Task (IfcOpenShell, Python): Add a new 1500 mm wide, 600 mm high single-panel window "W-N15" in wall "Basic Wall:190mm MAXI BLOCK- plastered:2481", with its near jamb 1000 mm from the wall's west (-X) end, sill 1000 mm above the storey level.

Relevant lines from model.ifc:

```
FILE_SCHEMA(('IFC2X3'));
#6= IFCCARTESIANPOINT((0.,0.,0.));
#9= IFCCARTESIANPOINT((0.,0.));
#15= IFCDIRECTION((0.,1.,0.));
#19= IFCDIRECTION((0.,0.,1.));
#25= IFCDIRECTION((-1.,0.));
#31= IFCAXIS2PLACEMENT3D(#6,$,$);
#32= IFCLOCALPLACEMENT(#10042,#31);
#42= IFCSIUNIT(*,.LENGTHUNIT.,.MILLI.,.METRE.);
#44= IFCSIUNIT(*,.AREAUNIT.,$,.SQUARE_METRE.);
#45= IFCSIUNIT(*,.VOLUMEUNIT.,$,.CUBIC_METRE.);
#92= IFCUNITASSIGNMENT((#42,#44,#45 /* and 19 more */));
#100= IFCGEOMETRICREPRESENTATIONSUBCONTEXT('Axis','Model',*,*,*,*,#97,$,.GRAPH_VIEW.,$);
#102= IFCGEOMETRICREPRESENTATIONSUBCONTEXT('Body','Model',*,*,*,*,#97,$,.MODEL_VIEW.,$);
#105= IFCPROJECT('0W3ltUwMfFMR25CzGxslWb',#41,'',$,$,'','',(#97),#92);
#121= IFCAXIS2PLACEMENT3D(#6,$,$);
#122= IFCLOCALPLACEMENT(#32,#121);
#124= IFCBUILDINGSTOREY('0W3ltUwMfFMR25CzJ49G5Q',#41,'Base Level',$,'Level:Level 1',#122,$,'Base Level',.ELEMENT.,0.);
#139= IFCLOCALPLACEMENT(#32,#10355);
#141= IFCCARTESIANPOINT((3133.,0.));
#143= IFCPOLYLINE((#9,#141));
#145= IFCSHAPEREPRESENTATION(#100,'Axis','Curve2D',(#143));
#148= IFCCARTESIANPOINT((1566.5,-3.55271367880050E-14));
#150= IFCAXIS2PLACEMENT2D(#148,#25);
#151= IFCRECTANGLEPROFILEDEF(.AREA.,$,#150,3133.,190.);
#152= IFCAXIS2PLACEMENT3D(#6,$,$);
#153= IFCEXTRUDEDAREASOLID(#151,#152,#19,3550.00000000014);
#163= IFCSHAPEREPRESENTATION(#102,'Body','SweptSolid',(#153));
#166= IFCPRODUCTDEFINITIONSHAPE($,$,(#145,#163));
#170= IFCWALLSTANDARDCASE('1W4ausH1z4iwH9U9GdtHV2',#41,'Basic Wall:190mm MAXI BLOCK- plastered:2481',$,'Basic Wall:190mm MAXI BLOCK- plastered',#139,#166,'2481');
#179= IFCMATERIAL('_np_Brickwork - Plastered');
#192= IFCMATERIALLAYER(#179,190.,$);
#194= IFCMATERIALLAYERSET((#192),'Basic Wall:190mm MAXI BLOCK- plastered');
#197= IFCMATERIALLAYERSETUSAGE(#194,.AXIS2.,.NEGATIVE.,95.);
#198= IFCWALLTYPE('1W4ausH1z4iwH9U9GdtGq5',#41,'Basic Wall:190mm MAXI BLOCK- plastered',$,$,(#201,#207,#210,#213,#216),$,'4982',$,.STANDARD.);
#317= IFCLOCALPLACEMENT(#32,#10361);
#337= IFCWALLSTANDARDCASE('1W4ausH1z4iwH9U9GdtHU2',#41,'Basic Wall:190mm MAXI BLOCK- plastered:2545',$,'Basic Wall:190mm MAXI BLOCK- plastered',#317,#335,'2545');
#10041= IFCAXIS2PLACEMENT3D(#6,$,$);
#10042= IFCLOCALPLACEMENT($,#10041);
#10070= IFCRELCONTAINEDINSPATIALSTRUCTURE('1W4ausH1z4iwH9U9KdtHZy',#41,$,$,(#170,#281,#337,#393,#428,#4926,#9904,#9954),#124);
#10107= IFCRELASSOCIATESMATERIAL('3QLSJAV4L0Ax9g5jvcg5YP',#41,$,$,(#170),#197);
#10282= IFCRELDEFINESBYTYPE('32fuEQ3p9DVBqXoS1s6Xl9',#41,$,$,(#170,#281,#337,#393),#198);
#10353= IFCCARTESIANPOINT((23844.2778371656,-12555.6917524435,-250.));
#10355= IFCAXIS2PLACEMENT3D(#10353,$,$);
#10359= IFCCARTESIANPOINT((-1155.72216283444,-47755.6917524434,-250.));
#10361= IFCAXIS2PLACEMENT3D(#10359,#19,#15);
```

```python
import numpy as np
import ifcopenshell
import ifcopenshell.api.feature
import ifcopenshell.api.geometry
import ifcopenshell.api.root
import ifcopenshell.api.spatial
import ifcopenshell.api.type
import ifcopenshell.geom
import ifcopenshell.util.element
import ifcopenshell.util.placement
import ifcopenshell.util.representation
import ifcopenshell.util.shape
import ifcopenshell.util.unit

model = ifcopenshell.open("model.ifc")
unit_scale = ifcopenshell.util.unit.calculate_unit_scale(model)
settings = ifcopenshell.geom.settings()


def volume(element):
    """Net volume in cubic metres, openings subtracted."""
    shape = ifcopenshell.geom.create_shape(settings, element)
    return ifcopenshell.util.shape.get_volume(shape.geometry)


wall = model.by_guid("1W4ausH1z4iwH9U9GdtHV2")
storey = ifcopenshell.util.element.get_container(wall, ifc_class="IfcBuildingStorey")
context = ifcopenshell.util.representation.get_context(model, "Model", "Body", "MODEL_VIEW")
before = volume(wall)

width, height, from_end, sill = 1.5, 0.6, 1, 1  # metres

# The wall runs along its own X axis, and the end named is its -X end.
wall_shape = ifcopenshell.geom.create_shape(settings, wall)
x, y, z = ifcopenshell.util.shape.get_vertices(wall_shape.geometry).T
start = x.min() + from_end
face, thickness = float(y.min()), float(y.max() - y.min())
wall_matrix = ifcopenshell.util.placement.get_local_placement(wall.ObjectPlacement)
level = ifcopenshell.util.placement.get_local_placement(storey.ObjectPlacement)[2, 3]


def in_wall(x, y):
    """Placement at x, y metres in the wall's axes, at sill height."""
    matrix = wall_matrix.copy()
    matrix[:, 3] = wall_matrix @ np.array([x / unit_scale, y / unit_scale, 0.0, 1.0])
    matrix[2, 3] = level + sill / unit_scale
    return matrix


# Opening: a box that overshoots both wall faces by 50 mm.
opening = ifcopenshell.api.root.create_entity(model, ifc_class="IfcOpeningElement")
box = ifcopenshell.api.geometry.add_wall_representation(
    model, context=context, length=width, height=height, thickness=thickness + 0.1
)
ifcopenshell.api.geometry.assign_representation(model, product=opening, representation=box)
ifcopenshell.api.geometry.edit_object_placement(model, product=opening, matrix=in_wall(start, face - 0.05), is_si=False)
ifcopenshell.api.feature.add_feature(model, feature=opening, element=wall)

window = ifcopenshell.api.root.create_entity(model, ifc_class="IfcWindow", name="W-N15")
window.OverallWidth, window.OverallHeight = width / unit_scale, height / unit_scale
body = ifcopenshell.api.geometry.add_window_representation(
    model,
    context=context,
    overall_width=window.OverallWidth,
    overall_height=window.OverallHeight,
    partition_type="SINGLE_PANEL",
)
ifcopenshell.api.geometry.assign_representation(model, product=window, representation=body)
ifcopenshell.api.spatial.assign_container(model, products=[window], relating_structure=storey)
fills = ifcopenshell.api.feature.add_filling(model, opening=opening, element=window)
fills.OwnerHistory = window.OwnerHistory  # required in IFC2X3

# IFC2X3 keeps the operation on the window style.
style = ifcopenshell.api.root.create_entity(model, ifc_class="IfcWindowStyle", name="W-N15")
style.OperationType, style.ConstructionType = "SINGLE_PANEL", "NOTDEFINED"
style.ParameterTakesPrecedence = style.Sizeable = False
ifcopenshell.api.type.assign_type(model, related_objects=[window], relating_type=style)

# Centre the window in the wall's thickness.
ifcopenshell.api.geometry.edit_object_placement(model, product=window, matrix=in_wall(start, face), is_si=False)
window_shape = ifcopenshell.geom.create_shape(settings, window)
depth = ifcopenshell.util.shape.get_vertices(window_shape.geometry)[:, 1]
offset = face + thickness / 2 - (depth.min() + depth.max()) / 2
ifcopenshell.api.geometry.edit_object_placement(model, product=window, matrix=in_wall(start, offset), is_si=False)

after = volume(wall)

print(f"wall volume {before:.3f} -> {after:.3f} m3")

model.write("model_edited.ifc")
```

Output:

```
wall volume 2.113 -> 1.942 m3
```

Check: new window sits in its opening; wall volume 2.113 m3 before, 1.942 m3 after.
